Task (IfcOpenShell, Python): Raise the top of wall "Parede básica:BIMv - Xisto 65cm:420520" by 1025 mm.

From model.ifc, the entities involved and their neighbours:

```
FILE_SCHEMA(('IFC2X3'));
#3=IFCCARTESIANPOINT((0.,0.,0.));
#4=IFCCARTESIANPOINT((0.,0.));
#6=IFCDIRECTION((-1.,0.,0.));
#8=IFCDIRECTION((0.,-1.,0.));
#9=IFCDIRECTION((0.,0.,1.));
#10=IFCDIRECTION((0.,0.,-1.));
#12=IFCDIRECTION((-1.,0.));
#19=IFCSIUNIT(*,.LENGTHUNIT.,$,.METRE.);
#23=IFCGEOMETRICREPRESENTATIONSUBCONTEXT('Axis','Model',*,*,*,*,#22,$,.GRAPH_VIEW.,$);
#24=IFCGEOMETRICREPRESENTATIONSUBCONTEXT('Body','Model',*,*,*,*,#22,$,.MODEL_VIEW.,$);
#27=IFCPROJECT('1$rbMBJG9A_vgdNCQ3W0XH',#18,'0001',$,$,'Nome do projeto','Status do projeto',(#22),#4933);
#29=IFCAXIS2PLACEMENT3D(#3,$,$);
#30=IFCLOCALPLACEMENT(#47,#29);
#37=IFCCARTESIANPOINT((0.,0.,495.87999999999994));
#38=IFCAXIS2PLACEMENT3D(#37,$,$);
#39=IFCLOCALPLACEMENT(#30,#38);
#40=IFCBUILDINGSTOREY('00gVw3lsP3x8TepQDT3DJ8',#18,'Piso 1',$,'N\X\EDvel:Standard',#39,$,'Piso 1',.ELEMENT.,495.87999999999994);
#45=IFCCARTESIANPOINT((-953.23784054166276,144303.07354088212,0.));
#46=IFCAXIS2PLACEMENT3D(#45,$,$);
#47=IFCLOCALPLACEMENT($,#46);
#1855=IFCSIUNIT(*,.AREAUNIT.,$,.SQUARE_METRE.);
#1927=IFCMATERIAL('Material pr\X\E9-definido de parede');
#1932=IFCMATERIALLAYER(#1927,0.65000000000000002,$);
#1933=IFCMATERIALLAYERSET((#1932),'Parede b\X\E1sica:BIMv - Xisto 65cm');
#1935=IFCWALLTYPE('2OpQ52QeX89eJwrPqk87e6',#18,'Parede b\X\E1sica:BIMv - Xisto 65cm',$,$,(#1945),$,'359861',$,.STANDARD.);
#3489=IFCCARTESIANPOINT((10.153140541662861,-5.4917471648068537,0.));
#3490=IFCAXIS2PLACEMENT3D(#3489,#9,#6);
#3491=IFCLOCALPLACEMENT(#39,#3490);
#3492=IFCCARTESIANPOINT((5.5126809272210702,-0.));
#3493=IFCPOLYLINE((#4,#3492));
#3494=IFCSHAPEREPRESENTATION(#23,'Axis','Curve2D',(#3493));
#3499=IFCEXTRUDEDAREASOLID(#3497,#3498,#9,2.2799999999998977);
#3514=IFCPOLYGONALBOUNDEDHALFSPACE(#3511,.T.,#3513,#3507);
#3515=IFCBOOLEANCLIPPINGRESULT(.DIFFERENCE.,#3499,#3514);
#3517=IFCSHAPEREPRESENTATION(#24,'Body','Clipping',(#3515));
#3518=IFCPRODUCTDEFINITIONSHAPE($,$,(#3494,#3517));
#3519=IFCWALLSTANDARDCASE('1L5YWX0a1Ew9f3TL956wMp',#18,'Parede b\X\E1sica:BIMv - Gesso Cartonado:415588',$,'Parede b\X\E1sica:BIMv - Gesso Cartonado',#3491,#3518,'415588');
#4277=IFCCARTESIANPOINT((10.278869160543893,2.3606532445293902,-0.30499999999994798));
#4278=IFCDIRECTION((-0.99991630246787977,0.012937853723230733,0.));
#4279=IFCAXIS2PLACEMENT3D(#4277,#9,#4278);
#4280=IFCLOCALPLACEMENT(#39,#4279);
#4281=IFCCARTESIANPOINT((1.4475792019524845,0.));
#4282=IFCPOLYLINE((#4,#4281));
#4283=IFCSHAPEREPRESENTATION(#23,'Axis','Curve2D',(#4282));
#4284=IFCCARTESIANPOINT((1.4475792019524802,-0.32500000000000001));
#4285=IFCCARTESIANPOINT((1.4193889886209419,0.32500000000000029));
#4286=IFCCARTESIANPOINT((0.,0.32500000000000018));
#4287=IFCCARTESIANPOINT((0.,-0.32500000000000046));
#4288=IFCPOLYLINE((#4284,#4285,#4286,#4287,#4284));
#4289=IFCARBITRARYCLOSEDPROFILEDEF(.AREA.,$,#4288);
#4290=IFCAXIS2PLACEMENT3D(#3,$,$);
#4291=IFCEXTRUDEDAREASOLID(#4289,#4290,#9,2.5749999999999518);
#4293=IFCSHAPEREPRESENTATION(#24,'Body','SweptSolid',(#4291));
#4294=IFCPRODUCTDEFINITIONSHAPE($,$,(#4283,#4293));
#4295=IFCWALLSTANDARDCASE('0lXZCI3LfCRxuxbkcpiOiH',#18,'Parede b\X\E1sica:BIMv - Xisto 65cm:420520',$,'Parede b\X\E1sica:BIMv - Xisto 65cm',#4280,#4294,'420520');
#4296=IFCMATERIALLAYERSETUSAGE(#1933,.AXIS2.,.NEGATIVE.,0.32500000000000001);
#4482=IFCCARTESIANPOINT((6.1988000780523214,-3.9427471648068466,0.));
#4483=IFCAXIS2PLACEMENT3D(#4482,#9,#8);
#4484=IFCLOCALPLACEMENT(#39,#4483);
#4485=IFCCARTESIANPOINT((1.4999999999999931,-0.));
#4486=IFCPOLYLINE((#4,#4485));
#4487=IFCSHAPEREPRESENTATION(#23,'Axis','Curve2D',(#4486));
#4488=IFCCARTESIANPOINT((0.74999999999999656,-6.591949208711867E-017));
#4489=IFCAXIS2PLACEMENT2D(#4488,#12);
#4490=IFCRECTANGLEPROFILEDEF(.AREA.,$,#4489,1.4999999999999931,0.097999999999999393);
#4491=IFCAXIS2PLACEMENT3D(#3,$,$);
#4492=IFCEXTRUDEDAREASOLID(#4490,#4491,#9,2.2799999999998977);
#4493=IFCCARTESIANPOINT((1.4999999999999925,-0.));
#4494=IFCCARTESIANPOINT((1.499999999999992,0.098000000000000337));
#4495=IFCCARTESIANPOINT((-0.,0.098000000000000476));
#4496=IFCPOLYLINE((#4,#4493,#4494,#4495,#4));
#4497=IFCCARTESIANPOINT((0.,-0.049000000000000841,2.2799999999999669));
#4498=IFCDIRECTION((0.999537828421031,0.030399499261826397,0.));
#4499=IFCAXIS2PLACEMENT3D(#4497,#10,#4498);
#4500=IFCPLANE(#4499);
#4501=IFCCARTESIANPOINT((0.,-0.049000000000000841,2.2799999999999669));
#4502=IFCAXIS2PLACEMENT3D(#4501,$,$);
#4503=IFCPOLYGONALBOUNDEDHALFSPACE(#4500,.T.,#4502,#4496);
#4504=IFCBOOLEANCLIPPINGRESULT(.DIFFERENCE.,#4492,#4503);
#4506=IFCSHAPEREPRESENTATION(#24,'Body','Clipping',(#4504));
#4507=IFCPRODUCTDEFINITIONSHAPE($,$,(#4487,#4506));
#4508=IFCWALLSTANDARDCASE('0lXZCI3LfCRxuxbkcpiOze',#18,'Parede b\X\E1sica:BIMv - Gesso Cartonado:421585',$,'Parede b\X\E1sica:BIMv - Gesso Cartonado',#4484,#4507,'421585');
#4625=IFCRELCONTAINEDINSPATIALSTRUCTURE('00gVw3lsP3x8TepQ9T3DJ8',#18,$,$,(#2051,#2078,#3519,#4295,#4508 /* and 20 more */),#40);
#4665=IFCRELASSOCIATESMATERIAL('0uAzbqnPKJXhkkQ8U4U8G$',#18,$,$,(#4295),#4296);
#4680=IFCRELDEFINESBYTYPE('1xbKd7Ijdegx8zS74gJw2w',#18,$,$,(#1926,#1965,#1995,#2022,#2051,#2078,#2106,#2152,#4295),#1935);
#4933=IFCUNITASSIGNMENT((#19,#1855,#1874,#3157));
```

```python
import ifcopenshell
import ifcopenshell.geom
import ifcopenshell.util.representation
import ifcopenshell.util.shape

model = ifcopenshell.open("model.ifc")
settings = ifcopenshell.geom.settings()


def volume(element):
    """Net volume in cubic metres, openings subtracted."""
    shape = ifcopenshell.geom.create_shape(settings, element)
    return ifcopenshell.util.shape.get_volume(shape.geometry)


wall = model.by_guid("0lXZCI3LfCRxuxbkcpiOiH")
before = volume(wall)

body = ifcopenshell.util.representation.get_representation(wall, "Model", "Body")
solid = body.Items[0]
old_height = solid.Depth
solid.Depth += 1.025
after = volume(wall)

print(f"height {old_height:g} -> {solid.Depth:g}, volume {before:.3f} -> {after:.3f} m3")

model.write("model-out.ifc")
```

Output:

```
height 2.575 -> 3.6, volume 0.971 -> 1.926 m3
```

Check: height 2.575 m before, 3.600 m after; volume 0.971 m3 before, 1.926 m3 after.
